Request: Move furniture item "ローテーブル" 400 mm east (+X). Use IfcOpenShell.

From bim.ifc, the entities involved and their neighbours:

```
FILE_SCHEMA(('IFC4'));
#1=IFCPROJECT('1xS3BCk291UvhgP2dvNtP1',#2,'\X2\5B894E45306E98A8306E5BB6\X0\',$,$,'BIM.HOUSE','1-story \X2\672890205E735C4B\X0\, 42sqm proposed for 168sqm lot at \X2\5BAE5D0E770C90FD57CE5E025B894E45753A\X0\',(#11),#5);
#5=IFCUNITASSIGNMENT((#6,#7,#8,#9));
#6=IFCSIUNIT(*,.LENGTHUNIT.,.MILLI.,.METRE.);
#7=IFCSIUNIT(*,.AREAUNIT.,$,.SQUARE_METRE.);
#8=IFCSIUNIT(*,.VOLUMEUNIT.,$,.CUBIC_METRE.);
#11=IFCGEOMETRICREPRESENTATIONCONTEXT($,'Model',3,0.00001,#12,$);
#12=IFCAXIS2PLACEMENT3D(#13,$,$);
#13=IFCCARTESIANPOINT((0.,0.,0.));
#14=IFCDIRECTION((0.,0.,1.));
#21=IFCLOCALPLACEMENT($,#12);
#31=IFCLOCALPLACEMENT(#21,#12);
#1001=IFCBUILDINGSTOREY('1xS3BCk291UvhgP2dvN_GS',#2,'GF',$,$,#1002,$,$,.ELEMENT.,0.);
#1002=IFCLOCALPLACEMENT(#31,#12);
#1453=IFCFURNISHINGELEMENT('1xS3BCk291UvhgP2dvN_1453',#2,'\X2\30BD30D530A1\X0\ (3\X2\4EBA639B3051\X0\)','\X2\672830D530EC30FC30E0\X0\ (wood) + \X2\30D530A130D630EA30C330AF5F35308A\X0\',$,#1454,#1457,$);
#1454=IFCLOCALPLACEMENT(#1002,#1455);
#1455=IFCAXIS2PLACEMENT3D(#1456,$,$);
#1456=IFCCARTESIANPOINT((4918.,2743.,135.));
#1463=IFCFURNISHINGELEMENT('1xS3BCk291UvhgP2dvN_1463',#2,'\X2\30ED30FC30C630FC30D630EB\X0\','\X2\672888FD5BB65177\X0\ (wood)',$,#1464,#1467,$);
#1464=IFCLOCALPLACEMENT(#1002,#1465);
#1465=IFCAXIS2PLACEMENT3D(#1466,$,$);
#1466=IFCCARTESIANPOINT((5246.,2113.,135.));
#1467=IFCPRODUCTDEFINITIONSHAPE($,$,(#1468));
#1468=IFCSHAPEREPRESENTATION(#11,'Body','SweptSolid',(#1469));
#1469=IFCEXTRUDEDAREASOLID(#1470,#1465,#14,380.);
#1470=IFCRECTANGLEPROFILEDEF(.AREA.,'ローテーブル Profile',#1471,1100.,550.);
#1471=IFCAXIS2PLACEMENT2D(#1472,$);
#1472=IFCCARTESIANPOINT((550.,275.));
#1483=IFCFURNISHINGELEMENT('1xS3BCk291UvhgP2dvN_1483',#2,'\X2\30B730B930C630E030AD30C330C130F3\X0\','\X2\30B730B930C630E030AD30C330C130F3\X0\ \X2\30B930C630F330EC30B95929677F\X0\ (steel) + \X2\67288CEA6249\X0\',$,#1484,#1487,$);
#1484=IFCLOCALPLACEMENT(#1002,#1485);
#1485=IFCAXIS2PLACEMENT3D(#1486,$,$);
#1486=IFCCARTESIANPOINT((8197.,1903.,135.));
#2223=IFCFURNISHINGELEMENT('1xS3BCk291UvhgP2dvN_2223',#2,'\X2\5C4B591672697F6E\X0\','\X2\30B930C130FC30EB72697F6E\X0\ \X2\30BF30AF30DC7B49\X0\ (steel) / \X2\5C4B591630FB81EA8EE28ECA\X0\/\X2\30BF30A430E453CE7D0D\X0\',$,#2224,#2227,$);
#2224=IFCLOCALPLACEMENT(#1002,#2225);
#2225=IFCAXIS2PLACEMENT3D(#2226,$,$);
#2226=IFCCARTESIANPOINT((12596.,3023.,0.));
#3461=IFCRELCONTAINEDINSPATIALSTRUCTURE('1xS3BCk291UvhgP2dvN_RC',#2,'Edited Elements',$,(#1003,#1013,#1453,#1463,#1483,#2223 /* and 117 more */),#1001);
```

```python
import ifcopenshell
import ifcopenshell.api.geometry
import ifcopenshell.util.placement

model = ifcopenshell.open("bim.ifc")

item = model.by_guid("1xS3BCk291UvhgP2dvN_1463")
matrix = ifcopenshell.util.placement.get_local_placement(item.ObjectPlacement)
matrix[0, 3] += 400.0
ifcopenshell.api.geometry.edit_object_placement(model, product=item, matrix=matrix, is_si=False)

print(ifcopenshell.util.placement.get_local_placement(item.ObjectPlacement).round(3) + 0.0)

model.write("bim_edited.ifc")
```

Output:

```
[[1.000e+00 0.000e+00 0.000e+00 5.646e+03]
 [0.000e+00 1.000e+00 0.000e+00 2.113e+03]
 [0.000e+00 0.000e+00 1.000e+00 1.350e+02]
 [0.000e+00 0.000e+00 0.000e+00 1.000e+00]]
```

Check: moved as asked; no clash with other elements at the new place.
